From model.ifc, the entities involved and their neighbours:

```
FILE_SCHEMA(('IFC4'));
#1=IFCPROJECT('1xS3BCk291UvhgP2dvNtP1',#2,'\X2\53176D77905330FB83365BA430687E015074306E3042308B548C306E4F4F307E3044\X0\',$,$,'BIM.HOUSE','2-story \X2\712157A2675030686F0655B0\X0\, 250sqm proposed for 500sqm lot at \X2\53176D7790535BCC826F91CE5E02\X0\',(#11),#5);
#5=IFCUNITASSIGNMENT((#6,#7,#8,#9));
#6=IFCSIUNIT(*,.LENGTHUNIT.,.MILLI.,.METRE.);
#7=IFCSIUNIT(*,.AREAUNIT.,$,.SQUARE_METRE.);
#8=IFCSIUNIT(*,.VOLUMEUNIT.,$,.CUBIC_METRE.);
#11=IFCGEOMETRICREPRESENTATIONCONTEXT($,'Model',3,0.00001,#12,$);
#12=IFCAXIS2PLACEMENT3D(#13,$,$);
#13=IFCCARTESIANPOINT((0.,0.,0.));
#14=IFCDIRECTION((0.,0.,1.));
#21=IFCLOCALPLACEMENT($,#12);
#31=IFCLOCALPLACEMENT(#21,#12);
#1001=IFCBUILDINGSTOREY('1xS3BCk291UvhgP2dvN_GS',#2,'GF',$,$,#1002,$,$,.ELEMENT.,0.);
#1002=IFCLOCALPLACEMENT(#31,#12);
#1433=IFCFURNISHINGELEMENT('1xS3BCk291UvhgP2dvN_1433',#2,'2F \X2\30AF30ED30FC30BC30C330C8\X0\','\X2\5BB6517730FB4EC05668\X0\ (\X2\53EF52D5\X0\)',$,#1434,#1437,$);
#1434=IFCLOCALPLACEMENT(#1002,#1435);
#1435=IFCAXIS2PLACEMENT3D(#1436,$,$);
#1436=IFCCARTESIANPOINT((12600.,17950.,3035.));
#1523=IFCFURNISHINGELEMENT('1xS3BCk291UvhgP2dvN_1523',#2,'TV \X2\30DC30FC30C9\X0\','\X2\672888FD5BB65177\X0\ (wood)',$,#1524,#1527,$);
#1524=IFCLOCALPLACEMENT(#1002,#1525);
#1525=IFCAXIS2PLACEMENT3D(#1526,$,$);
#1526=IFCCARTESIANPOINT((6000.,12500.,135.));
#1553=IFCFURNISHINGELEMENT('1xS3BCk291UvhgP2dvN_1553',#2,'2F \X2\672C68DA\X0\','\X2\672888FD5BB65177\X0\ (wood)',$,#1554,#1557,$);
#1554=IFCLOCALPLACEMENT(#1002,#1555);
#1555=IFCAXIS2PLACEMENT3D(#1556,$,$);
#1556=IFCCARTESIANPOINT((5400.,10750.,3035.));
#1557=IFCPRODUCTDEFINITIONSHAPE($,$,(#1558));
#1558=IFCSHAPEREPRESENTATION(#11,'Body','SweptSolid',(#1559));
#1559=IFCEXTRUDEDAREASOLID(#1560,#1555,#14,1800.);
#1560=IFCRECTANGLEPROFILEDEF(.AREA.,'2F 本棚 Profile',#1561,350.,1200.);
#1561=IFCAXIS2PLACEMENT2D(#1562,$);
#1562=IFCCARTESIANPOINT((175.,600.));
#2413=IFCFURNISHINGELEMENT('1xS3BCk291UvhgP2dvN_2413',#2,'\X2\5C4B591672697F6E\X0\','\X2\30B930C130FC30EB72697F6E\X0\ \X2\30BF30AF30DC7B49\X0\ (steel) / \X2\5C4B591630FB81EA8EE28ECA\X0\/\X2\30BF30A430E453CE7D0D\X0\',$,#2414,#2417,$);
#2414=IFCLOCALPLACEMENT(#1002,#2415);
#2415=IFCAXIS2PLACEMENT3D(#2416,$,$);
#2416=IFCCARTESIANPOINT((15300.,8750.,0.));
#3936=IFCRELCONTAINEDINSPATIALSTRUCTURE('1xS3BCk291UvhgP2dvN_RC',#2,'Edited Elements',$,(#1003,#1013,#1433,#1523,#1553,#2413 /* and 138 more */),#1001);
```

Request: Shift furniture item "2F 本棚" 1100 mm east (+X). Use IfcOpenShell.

```python
import ifcopenshell
import ifcopenshell.api.geometry
import ifcopenshell.util.placement
import ifcopenshell.util.unit

model = ifcopenshell.open("model.ifc")
unit_scale = ifcopenshell.util.unit.calculate_unit_scale(model)

item = model.by_guid("1xS3BCk291UvhgP2dvN_1553")
matrix = ifcopenshell.util.placement.get_local_placement(item.ObjectPlacement)
matrix[0, 3] += 1.1 / unit_scale
ifcopenshell.api.geometry.edit_object_placement(model, product=item, matrix=matrix, is_si=False)

print(ifcopenshell.util.placement.get_local_placement(item.ObjectPlacement).round(3) + 0.0)

model.write("model-out.ifc")
```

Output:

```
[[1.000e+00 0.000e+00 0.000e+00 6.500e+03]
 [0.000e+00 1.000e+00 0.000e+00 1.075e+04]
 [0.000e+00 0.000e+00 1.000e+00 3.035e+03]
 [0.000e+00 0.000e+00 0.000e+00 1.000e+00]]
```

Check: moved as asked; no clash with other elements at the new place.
